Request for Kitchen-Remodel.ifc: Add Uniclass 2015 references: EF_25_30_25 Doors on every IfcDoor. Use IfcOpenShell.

First a look at what the model holds.

```python
import ifcopenshell

model = ifcopenshell.open("Kitchen-Remodel.ifc")
print(model.schema)
print("classifications:", [c.Name for c in model.by_type("IfcClassification")])
for ifc_class in ("IfcDoor", "IfcRoof", "IfcStair", "IfcWall", "IfcWindow"):
    print(ifc_class, len(model.by_type(ifc_class)))
```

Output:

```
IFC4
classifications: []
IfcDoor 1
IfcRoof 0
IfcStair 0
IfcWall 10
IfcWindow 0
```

```python
import ifcopenshell
import ifcopenshell.api.classification

model = ifcopenshell.open("Kitchen-Remodel.ifc")

system = ifcopenshell.api.classification.add_classification(model, classification="Uniclass 2015")

codes = {
    "IfcDoor": ("EF_25_30_25", "Doors"),
}
for ifc_class, (code, name) in codes.items():
    products = model.by_type(ifc_class)
    ifcopenshell.api.classification.add_reference(
        model, products=products, classification=system, identification=code, name=name
    )
    print(code, len(products))

model.write("Kitchen-Remodel-out.ifc")
```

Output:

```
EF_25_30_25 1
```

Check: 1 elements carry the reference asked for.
